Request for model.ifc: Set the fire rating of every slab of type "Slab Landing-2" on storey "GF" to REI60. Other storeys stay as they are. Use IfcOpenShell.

First a look at what the model holds.

```python
import ifcopenshell
import ifcopenshell.util.element

model = ifcopenshell.open("model.ifc")
print(model.schema)
storey = next(s for s in model.by_type("IfcBuildingStorey") if s.Name == "GF")
slabs = [e for e in ifcopenshell.util.element.get_decomposition(storey) if e.is_a("IfcSlab")]
seen = {}
for e in slabs:
    element_type = ifcopenshell.util.element.get_type(e)
    key = (element_type.Name if element_type != e and element_type else None, ifcopenshell.util.element.get_pset(e, "Pset_SlabCommon", "FireRating"))
    seen[key] = seen.get(key, 0) + 1
for (name, value), count in sorted(seen.items(), key=str):
    print(count, "x", name, "|", value)
```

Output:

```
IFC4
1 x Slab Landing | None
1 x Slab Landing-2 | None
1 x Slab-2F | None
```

```python
import ifcopenshell
import ifcopenshell.api.pset
import ifcopenshell.util.element

model = ifcopenshell.open("model.ifc")

storey = next(s for s in model.by_type("IfcBuildingStorey") if s.Name == "GF")
slabs = [e for e in ifcopenshell.util.element.get_decomposition(storey) if e.is_a("IfcSlab")]

count = 0
for e in slabs:
    element_type = ifcopenshell.util.element.get_type(e)
    if element_type in (None, e) or element_type.Name != "Slab Landing-2":
        continue
    # add_pset returns the element's existing set when there is one.
    pset = ifcopenshell.api.pset.add_pset(model, product=e, name="Pset_SlabCommon")
    ifcopenshell.api.pset.edit_pset(model, pset=pset, properties={"FireRating": "REI60"})
    count += 1

print(count, "slabs updated")

model.write("model_v2.ifc")
```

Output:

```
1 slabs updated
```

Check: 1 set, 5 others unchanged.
